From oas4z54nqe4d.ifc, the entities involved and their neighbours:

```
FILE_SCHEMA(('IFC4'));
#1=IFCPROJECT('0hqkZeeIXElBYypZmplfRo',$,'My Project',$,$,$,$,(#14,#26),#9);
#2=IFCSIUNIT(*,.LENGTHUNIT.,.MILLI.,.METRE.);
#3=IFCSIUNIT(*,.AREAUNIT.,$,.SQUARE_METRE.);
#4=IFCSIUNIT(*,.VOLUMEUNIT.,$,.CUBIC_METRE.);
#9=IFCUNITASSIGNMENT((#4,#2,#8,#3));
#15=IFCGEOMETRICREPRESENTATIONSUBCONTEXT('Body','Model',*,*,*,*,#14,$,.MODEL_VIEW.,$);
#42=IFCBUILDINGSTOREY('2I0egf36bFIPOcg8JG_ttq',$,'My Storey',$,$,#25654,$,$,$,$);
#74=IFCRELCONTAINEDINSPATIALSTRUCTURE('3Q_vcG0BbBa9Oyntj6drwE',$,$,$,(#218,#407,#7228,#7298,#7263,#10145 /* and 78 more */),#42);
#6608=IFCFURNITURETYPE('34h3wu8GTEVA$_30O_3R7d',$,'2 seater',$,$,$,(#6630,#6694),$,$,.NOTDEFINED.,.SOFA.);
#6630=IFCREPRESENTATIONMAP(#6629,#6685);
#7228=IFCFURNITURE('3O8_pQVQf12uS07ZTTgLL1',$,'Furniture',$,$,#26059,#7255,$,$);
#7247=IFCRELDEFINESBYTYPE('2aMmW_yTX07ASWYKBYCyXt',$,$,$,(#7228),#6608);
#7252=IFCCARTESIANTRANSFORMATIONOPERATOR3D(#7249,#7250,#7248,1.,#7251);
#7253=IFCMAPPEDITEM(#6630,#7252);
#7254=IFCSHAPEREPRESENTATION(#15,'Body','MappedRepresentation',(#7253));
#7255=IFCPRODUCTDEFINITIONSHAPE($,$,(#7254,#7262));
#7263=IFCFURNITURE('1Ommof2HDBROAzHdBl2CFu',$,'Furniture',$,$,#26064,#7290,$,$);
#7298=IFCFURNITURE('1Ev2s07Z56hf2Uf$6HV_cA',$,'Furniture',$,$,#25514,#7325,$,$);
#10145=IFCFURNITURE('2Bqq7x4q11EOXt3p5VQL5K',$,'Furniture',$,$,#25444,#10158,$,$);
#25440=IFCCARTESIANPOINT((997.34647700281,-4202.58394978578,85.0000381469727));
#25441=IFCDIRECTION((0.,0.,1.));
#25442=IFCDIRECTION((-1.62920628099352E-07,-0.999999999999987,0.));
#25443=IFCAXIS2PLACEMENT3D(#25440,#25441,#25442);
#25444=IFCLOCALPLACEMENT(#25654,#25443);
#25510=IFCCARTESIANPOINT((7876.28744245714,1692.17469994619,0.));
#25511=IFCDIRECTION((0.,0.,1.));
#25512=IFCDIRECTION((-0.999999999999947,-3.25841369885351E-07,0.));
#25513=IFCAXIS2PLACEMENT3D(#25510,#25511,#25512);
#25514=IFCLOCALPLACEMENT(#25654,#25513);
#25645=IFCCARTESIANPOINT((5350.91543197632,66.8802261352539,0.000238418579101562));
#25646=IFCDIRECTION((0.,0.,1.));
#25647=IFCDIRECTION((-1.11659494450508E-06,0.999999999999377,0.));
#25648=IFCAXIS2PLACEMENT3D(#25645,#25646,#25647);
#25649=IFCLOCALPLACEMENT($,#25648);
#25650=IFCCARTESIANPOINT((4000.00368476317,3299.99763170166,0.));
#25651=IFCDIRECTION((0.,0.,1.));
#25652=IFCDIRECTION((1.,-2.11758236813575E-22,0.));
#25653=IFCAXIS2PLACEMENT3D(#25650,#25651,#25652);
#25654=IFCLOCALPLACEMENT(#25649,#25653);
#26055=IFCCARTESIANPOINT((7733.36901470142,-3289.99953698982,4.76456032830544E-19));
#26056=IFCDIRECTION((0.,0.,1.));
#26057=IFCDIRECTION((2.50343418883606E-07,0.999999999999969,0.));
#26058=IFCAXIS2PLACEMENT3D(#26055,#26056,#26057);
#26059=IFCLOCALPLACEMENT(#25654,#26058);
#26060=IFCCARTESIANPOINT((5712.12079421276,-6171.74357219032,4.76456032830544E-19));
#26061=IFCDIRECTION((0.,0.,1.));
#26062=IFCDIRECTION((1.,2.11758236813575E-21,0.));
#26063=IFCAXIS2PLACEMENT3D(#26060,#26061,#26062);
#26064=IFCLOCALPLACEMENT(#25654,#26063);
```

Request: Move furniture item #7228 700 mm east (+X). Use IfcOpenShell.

```python
import ifcopenshell
import ifcopenshell.api.geometry
import ifcopenshell.util.placement
import ifcopenshell.util.unit

model = ifcopenshell.open("oas4z54nqe4d.ifc")
unit_scale = ifcopenshell.util.unit.calculate_unit_scale(model)

item = model.by_guid("3O8_pQVQf12uS07ZTTgLL1")
matrix = ifcopenshell.util.placement.get_local_placement(item.ObjectPlacement)
matrix[0, 3] += 0.7 / unit_scale
ifcopenshell.api.geometry.edit_object_placement(model, product=item, matrix=matrix, is_si=False)

print(ifcopenshell.util.placement.get_local_placement(item.ObjectPlacement).round(3) + 0.0)

model.write("oas4z54nqe4d_updated.ifc")
```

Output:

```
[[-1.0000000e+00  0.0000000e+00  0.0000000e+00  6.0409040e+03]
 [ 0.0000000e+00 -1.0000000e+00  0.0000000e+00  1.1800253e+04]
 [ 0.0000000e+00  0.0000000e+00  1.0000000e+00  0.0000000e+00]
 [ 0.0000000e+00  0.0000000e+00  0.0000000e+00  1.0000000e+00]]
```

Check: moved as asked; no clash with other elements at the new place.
